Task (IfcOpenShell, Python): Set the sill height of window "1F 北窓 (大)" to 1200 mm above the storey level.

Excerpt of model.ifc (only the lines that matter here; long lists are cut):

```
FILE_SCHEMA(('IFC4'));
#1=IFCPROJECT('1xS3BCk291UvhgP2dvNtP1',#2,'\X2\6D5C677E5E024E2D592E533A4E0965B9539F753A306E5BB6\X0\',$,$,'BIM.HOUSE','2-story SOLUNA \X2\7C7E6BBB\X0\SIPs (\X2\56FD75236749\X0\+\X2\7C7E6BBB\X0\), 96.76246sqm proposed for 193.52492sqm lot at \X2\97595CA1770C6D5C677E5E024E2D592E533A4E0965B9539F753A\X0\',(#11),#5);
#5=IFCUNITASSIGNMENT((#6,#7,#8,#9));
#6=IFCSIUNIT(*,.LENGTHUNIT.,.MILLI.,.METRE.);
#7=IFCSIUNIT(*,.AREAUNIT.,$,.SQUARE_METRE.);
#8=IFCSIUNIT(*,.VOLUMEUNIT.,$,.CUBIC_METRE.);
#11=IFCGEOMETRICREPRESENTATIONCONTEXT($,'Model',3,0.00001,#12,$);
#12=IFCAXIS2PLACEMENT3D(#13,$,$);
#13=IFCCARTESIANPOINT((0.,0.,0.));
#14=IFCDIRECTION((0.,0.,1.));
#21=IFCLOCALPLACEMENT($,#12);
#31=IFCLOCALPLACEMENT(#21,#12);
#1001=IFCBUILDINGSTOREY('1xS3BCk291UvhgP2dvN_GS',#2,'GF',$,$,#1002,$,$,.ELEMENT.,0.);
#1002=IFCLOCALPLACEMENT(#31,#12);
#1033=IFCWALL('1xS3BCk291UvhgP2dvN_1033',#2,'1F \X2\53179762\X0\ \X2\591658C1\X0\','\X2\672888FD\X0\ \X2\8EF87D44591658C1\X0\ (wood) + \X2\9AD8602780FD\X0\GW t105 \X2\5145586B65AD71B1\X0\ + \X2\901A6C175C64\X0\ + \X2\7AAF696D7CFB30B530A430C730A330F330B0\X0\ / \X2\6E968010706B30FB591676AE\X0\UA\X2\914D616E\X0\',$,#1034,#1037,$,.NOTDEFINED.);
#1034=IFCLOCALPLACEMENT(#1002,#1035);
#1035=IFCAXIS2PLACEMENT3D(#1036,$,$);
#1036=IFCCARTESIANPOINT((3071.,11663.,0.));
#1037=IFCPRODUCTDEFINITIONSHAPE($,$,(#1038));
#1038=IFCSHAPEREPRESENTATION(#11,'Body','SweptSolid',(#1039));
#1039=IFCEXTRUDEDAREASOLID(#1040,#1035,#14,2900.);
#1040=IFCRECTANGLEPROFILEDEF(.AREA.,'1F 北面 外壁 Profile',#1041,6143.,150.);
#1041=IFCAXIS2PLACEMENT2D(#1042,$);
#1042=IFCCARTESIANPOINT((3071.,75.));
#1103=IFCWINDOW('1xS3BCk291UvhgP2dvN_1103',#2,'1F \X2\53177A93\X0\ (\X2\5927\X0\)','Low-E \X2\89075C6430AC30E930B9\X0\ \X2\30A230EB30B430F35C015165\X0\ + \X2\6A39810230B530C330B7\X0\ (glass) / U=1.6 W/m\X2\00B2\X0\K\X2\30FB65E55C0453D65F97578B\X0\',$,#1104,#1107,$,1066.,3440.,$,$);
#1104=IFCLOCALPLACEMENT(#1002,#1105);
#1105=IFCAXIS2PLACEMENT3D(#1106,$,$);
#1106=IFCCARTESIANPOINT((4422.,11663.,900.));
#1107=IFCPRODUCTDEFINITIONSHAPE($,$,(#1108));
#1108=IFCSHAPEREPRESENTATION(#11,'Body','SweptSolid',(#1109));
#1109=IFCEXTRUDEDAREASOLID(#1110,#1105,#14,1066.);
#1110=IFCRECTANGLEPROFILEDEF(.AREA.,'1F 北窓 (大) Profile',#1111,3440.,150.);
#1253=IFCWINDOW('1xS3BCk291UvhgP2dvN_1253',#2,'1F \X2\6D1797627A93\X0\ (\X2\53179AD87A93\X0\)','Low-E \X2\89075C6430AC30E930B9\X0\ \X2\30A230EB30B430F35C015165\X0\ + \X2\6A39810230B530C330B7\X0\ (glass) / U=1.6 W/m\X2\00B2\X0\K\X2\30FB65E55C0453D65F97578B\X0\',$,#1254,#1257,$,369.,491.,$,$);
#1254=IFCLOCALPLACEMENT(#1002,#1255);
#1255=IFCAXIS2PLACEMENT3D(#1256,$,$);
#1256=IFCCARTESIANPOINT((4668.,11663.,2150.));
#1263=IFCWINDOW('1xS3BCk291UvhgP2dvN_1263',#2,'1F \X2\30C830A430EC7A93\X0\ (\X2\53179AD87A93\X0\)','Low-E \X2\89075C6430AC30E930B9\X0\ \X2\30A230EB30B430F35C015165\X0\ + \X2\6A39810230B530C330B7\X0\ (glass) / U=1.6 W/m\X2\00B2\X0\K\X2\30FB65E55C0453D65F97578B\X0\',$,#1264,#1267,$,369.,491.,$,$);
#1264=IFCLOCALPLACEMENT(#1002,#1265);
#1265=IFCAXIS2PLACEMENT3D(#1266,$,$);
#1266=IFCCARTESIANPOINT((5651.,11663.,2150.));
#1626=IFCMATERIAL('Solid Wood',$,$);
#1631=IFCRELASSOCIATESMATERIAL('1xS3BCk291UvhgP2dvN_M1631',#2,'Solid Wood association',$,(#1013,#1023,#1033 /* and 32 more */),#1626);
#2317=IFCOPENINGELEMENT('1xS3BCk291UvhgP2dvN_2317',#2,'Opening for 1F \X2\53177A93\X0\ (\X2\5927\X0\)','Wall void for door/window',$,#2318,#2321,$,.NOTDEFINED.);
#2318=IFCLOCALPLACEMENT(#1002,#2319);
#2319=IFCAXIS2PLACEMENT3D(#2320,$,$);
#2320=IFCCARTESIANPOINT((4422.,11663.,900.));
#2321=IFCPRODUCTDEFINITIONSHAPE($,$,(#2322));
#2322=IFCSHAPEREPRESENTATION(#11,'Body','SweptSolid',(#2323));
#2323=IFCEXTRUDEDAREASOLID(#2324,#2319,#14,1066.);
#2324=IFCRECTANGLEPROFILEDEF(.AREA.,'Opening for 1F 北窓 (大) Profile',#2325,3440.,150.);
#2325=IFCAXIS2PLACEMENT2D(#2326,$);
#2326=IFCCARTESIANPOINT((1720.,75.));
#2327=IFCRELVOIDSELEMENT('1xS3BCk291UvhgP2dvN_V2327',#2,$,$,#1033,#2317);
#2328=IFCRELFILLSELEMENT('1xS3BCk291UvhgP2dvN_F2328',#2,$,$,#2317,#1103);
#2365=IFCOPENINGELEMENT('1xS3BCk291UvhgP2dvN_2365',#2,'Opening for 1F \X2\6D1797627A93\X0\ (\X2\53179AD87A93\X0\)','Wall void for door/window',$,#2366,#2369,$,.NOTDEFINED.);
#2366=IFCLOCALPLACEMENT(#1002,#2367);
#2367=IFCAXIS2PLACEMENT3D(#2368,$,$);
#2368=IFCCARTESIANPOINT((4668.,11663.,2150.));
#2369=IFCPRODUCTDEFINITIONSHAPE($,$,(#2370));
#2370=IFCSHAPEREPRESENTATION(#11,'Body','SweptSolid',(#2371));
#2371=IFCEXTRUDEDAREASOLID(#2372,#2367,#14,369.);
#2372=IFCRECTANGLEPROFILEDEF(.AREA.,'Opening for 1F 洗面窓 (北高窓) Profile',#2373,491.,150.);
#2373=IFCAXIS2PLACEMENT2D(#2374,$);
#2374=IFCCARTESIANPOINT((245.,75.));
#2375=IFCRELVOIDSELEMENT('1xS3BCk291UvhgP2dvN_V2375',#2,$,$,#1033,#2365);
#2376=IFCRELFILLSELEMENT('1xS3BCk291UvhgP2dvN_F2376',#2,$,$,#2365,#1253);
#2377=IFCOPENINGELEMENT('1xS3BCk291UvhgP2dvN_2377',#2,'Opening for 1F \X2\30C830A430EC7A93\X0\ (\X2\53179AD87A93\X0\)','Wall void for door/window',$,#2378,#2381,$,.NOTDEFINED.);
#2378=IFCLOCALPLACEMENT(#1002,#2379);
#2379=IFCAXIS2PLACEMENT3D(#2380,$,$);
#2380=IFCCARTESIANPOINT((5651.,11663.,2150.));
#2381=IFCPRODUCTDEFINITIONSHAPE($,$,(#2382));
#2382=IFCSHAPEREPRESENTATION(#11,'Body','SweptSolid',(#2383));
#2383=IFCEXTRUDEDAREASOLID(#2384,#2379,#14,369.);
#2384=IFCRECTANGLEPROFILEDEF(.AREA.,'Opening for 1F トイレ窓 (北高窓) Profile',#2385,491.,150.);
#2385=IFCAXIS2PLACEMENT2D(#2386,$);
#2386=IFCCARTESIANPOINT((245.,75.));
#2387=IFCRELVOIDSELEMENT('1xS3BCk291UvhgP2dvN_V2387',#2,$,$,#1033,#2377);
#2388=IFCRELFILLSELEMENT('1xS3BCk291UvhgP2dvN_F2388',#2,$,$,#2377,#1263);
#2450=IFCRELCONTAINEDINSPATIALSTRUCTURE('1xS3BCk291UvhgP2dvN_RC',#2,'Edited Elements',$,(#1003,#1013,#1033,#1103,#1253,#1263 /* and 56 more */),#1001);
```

```python
import numpy as np
import ifcopenshell
import ifcopenshell.api.geometry
import ifcopenshell.geom
import ifcopenshell.util.element
import ifcopenshell.util.placement
import ifcopenshell.util.shape
import ifcopenshell.util.unit

model = ifcopenshell.open("model.ifc")
unit_scale = ifcopenshell.util.unit.calculate_unit_scale(model)

window = model.by_guid("1xS3BCk291UvhgP2dvN_1103")
opening = window.FillsVoids[0].RelatingOpeningElement
storey = ifcopenshell.util.element.get_container(window, ifc_class="IfcBuildingStorey")
level = ifcopenshell.util.placement.get_local_placement(storey.ObjectPlacement)[2, 3]

# The opening's origin need not be at the sill, so measure its lowest point.
shape = ifcopenshell.geom.create_shape(ifcopenshell.geom.settings(), opening)
bottom = ifcopenshell.util.shape.get_shape_bottom_elevation(shape, shape.geometry) / unit_scale
dz = level + 1200.0 - bottom

shift = np.array([0.0, 0.0, dz])
# The window is not placed relative to its opening, so move both.
for product in (opening, window):
    matrix = ifcopenshell.util.placement.get_local_placement(product.ObjectPlacement)
    matrix[:3, 3] += shift
    ifcopenshell.api.geometry.edit_object_placement(model, product=product, matrix=matrix, is_si=False)

print(f"moved by {dz * unit_scale:+.3f} m")

model.write("model_v2.ifc")
```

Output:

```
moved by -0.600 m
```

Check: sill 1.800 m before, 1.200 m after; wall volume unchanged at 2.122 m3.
